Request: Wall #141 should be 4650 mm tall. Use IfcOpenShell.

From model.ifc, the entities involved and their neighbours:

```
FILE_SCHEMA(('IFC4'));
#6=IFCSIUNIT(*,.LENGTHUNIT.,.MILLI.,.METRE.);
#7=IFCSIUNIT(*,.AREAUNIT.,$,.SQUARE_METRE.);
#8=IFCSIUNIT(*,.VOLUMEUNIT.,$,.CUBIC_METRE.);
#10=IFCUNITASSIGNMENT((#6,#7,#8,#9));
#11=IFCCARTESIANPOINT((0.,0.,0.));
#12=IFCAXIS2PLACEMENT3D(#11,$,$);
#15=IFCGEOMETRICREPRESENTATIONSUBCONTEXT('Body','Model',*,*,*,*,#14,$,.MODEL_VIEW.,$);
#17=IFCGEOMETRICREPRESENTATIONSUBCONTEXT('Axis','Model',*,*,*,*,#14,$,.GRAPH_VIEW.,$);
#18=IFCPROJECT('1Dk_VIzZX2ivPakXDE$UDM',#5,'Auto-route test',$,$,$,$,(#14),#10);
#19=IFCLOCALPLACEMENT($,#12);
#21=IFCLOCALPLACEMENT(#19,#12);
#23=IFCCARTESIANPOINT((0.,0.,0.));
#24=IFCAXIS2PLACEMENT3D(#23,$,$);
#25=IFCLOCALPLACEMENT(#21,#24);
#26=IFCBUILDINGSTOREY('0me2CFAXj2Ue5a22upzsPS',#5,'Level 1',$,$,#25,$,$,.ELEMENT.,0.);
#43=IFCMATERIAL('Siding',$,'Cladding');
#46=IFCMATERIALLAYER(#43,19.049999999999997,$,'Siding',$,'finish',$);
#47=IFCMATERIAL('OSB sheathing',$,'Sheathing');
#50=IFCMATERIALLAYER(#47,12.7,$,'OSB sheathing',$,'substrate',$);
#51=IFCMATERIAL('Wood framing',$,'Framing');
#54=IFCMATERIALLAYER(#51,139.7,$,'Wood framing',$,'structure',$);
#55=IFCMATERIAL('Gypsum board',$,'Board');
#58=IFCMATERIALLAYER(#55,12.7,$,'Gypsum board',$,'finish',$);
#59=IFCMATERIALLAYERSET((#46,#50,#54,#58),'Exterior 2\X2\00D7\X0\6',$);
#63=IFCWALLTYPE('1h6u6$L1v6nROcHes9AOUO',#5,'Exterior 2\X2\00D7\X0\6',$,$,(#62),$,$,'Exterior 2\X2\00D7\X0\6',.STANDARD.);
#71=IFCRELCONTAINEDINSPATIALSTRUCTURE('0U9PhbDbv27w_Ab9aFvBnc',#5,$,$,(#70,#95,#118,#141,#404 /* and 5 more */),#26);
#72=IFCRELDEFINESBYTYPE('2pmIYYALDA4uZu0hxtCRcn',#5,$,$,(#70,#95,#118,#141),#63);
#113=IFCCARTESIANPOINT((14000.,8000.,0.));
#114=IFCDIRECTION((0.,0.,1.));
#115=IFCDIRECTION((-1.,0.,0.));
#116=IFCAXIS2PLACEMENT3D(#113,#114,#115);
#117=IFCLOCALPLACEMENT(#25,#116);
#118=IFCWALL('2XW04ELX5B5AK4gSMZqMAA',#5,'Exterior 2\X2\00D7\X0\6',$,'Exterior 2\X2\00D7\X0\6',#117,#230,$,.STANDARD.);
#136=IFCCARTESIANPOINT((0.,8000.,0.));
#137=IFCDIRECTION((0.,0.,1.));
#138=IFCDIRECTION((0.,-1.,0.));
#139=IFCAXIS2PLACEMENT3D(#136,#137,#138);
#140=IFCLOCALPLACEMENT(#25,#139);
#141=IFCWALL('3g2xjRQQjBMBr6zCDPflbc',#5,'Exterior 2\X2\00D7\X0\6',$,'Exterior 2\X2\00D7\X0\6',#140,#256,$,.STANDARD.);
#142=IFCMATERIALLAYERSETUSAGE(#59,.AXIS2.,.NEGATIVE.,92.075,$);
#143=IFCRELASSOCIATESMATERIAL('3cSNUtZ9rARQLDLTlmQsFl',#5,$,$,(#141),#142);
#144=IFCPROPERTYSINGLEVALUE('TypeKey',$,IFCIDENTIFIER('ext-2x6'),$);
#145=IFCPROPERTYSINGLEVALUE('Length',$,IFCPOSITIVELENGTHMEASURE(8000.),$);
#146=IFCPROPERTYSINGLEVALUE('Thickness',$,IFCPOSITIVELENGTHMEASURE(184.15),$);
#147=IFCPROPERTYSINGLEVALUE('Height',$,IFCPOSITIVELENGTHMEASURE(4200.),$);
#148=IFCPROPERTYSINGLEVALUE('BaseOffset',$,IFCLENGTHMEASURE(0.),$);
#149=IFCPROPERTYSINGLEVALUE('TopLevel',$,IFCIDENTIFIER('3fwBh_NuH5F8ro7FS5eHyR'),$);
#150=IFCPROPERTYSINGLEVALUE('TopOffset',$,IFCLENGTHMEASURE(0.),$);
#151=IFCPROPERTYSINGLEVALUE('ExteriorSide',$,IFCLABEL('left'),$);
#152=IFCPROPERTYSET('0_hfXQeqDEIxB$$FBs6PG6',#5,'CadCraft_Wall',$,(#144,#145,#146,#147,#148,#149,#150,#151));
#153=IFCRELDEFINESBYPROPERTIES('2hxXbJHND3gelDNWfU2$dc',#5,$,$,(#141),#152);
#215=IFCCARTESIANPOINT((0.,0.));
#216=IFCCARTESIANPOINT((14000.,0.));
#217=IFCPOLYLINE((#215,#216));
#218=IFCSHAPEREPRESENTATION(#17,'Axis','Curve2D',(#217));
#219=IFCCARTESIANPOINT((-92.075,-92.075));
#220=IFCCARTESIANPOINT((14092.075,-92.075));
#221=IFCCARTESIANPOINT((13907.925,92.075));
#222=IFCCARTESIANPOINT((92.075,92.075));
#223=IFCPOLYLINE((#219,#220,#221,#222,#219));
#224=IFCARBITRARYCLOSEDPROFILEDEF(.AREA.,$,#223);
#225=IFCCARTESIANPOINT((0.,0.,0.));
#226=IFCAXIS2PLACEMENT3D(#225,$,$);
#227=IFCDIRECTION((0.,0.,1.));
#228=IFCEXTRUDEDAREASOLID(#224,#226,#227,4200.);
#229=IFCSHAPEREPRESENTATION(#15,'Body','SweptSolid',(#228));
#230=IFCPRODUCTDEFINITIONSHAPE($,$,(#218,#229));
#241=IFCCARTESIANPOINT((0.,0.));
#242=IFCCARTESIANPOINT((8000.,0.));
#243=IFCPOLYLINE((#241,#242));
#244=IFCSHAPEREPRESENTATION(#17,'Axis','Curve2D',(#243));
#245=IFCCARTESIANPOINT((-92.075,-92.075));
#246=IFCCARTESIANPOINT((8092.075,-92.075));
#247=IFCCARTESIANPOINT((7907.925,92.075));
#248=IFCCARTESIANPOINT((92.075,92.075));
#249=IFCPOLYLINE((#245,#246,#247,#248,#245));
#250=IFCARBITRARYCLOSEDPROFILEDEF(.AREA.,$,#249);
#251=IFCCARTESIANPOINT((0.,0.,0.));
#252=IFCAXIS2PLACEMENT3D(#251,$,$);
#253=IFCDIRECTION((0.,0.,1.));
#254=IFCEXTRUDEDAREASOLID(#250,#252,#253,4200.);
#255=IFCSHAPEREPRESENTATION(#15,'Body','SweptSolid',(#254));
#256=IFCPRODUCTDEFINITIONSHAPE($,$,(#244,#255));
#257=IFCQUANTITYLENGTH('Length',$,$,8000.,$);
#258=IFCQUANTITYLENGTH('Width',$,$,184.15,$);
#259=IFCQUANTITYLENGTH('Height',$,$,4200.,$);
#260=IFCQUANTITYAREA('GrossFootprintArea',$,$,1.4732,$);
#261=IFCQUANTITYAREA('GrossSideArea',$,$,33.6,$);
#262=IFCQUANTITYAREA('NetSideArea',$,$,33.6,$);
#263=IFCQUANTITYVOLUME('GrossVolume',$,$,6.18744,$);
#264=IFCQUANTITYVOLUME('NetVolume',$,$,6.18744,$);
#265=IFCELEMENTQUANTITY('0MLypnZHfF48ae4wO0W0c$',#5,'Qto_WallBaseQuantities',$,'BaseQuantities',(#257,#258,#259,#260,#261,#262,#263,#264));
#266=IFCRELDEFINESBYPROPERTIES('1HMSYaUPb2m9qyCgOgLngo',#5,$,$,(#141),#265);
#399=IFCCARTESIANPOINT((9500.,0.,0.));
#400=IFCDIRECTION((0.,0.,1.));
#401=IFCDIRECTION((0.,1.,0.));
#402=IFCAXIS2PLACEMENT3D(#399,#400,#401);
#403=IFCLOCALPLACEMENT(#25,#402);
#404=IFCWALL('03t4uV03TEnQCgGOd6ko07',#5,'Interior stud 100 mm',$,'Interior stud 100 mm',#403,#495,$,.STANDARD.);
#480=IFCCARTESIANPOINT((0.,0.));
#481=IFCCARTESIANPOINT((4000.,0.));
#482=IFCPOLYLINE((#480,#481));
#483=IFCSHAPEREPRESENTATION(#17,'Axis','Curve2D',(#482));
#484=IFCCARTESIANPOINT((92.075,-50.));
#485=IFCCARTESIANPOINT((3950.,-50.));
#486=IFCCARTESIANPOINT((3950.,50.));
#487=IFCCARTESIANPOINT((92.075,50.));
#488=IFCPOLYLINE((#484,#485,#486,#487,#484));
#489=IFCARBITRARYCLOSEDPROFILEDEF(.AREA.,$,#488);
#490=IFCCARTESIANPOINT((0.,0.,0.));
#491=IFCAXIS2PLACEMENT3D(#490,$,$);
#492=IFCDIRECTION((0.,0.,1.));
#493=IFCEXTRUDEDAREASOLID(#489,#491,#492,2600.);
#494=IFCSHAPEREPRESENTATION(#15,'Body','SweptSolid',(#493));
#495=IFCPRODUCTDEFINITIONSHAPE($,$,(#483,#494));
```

```python
import ifcopenshell
import ifcopenshell.api.pset
import ifcopenshell.geom
import ifcopenshell.util.element
import ifcopenshell.util.representation
import ifcopenshell.util.shape
import ifcopenshell.util.unit

model = ifcopenshell.open("model.ifc")
unit_scale = ifcopenshell.util.unit.calculate_unit_scale(model)
area_scale = ifcopenshell.util.unit.calculate_unit_scale(model, "AREAUNIT")
volume_scale = ifcopenshell.util.unit.calculate_unit_scale(model, "VOLUMEUNIT")
settings = ifcopenshell.geom.settings()


def volume(element):
    """Net volume in cubic metres, openings subtracted."""
    shape = ifcopenshell.geom.create_shape(settings, element)
    return ifcopenshell.util.shape.get_volume(shape.geometry)


wall = model.by_guid("3g2xjRQQjBMBr6zCDPflbc")
before = volume(wall)

body = ifcopenshell.util.representation.get_representation(wall, "Model", "Body")
solid = body.Items[0]
old_height = solid.Depth
solid.Depth = 4.65 / unit_scale
after = volume(wall)
thickness = 0.1842  # wall thickness in metres

# Update the stored height, areas and volumes.
pset = model.by_id(ifcopenshell.util.element.get_pset(wall, "CadCraft_Wall", should_inherit=False)["id"])
ifcopenshell.api.pset.edit_pset(model, pset=pset, properties={
    "Height": model.create_entity("IfcPositiveLengthMeasure", solid.Depth),
})
qto = model.by_id(ifcopenshell.util.element.get_pset(wall, "Qto_WallBaseQuantities", should_inherit=False)["id"])
ifcopenshell.api.pset.edit_qto(model, qto=qto, properties={
    "Height": solid.Depth,
    "GrossSideArea": ifcopenshell.util.element.get_pset(wall, "Qto_WallBaseQuantities", "GrossSideArea") * solid.Depth / old_height,
    "NetSideArea": after / thickness / area_scale,
    "GrossVolume": ifcopenshell.util.element.get_pset(wall, "Qto_WallBaseQuantities", "GrossVolume") * solid.Depth / old_height,
    "NetVolume": after / volume_scale,
})

print(f"height {old_height:g} -> {solid.Depth:g}, volume {before:.3f} -> {after:.3f} m3")

model.write("model_updated.ifc")
```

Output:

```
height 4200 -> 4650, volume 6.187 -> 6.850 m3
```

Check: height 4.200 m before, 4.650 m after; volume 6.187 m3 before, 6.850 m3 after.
